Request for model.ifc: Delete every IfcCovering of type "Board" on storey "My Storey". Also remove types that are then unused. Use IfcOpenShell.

First a look at what the model holds.

```python
import ifcopenshell
import ifcopenshell.util.element

model = ifcopenshell.open("model.ifc")
print(model.schema)
storey = next(s for s in model.by_type("IfcBuildingStorey") if s.Name == "My Storey")
coverings = [e for e in ifcopenshell.util.element.get_decomposition(storey) if e.is_a("IfcCovering")]
seen = {}
for e in coverings:
    element_type = ifcopenshell.util.element.get_type(e)
    name = element_type.Name if element_type not in (None, e) else None
    seen[name] = seen.get(name, 0) + 1
for name, count in sorted(seen.items(), key=str):
    print(count, "x", name)
```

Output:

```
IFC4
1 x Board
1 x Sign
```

```python
import ifcopenshell
import ifcopenshell.api.root
import ifcopenshell.util.element

model = ifcopenshell.open("model.ifc")

storey = next(s for s in model.by_type("IfcBuildingStorey") if s.Name == "My Storey")
coverings = [e for e in ifcopenshell.util.element.get_decomposition(storey) if e.is_a("IfcCovering")]
targets = [e for e in coverings if (t := ifcopenshell.util.element.get_type(e)) not in (None, e) and t.Name == "Board"]
types = {ifcopenshell.util.element.get_type(e) for e in targets} - {None, *targets}

for e in targets:
    ifcopenshell.api.root.remove_product(model, product=e)
print(len(targets), "removed")

unused = [t for t in types if not ifcopenshell.util.element.get_types(t)]
for t in unused:
    ifcopenshell.api.root.remove_product(model, product=t)
print(len(unused), "unused types removed")

model.write("model_rev.ifc")
```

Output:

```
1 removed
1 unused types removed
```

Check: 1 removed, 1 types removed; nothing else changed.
